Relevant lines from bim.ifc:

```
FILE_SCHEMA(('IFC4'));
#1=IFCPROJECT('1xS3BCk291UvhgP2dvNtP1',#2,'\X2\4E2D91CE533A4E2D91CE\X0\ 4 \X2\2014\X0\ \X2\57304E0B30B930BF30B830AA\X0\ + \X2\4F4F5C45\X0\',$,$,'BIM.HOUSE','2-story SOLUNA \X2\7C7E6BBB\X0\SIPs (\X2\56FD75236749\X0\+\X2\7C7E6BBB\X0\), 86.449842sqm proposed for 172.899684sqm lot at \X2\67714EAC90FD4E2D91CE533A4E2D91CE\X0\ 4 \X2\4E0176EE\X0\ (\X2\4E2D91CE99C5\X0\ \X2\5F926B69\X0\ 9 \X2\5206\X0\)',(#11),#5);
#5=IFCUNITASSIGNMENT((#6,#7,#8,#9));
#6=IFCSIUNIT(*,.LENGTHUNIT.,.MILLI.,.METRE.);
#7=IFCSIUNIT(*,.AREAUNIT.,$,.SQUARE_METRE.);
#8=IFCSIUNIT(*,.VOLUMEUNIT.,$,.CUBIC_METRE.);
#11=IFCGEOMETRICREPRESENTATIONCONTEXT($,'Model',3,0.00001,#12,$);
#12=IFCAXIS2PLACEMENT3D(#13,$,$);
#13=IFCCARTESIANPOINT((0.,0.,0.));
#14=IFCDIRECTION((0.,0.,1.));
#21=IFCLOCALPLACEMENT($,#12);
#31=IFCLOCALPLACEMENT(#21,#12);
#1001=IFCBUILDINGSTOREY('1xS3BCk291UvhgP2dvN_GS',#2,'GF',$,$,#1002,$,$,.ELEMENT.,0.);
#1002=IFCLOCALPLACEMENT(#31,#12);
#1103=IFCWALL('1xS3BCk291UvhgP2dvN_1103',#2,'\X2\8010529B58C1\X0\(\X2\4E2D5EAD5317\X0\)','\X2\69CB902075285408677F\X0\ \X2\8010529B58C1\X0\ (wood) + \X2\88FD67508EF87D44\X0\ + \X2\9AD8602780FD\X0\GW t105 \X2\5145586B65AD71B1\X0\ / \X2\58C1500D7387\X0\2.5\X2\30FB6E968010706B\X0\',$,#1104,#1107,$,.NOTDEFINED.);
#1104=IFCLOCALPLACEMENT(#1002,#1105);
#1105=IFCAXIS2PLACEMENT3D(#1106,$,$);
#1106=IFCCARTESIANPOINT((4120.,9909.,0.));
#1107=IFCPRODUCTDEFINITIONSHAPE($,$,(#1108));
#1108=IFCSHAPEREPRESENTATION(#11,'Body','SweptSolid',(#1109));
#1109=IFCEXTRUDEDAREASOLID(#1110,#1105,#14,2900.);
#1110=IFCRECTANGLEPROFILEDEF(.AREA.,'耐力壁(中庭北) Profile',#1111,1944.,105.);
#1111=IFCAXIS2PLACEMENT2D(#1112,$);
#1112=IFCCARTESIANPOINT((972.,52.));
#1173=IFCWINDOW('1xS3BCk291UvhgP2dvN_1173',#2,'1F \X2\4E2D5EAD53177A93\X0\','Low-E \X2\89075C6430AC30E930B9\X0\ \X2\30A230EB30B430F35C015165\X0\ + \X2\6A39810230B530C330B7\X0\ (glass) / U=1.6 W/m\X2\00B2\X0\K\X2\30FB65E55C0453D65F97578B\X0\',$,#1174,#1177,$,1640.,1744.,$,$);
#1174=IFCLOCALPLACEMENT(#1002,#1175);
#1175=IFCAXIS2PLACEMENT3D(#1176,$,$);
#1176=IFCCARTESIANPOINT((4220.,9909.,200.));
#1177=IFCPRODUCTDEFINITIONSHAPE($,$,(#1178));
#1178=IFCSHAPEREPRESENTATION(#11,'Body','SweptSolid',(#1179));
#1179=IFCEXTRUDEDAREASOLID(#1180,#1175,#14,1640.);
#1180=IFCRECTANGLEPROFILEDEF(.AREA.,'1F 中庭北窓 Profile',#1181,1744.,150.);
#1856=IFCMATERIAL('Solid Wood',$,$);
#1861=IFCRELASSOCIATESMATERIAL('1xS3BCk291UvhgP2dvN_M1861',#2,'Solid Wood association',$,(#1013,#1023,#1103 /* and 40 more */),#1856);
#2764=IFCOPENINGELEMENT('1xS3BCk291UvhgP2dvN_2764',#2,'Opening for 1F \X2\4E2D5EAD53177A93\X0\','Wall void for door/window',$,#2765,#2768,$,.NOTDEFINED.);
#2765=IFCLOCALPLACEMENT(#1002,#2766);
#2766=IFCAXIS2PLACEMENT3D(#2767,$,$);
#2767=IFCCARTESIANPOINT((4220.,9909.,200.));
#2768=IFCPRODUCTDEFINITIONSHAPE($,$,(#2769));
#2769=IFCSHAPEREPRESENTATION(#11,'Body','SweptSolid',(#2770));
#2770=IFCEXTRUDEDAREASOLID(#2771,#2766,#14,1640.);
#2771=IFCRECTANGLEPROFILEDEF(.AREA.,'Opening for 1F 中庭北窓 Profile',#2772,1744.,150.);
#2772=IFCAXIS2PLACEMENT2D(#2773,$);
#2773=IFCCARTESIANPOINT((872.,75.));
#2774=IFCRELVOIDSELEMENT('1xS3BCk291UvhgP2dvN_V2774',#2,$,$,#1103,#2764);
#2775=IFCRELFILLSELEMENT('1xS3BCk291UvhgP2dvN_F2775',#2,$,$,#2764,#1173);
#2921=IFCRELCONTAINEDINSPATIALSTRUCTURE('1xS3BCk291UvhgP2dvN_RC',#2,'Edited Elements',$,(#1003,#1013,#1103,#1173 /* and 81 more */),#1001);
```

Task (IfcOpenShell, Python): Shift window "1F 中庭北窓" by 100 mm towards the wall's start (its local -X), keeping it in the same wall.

```python
import ifcopenshell
import ifcopenshell.api.geometry
import ifcopenshell.util.placement

model = ifcopenshell.open("bim.ifc")

window = model.by_guid("1xS3BCk291UvhgP2dvN_1173")
opening = window.FillsVoids[0].RelatingOpeningElement
wall = opening.VoidsElements[0].RelatingBuildingElement

wall_matrix = ifcopenshell.util.placement.get_local_placement(wall.ObjectPlacement)
shift = wall_matrix[:3, 0] * -100.0
before = ifcopenshell.util.placement.get_local_placement(window.ObjectPlacement)[:3, 3].copy()

# The window is not placed relative to its opening, so move both.
for product in (opening, window):
    matrix = ifcopenshell.util.placement.get_local_placement(product.ObjectPlacement)
    matrix[:3, 3] += shift
    ifcopenshell.api.geometry.edit_object_placement(model, product=product, matrix=matrix, is_si=False)

after = ifcopenshell.util.placement.get_local_placement(window.ObjectPlacement)[:3, 3]
print("window moved by", (after - before).round(3) + 0.0)

model.write("bim_rev.ifc")
```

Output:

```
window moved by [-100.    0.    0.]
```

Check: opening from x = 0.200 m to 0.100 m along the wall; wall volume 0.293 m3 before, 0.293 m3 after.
